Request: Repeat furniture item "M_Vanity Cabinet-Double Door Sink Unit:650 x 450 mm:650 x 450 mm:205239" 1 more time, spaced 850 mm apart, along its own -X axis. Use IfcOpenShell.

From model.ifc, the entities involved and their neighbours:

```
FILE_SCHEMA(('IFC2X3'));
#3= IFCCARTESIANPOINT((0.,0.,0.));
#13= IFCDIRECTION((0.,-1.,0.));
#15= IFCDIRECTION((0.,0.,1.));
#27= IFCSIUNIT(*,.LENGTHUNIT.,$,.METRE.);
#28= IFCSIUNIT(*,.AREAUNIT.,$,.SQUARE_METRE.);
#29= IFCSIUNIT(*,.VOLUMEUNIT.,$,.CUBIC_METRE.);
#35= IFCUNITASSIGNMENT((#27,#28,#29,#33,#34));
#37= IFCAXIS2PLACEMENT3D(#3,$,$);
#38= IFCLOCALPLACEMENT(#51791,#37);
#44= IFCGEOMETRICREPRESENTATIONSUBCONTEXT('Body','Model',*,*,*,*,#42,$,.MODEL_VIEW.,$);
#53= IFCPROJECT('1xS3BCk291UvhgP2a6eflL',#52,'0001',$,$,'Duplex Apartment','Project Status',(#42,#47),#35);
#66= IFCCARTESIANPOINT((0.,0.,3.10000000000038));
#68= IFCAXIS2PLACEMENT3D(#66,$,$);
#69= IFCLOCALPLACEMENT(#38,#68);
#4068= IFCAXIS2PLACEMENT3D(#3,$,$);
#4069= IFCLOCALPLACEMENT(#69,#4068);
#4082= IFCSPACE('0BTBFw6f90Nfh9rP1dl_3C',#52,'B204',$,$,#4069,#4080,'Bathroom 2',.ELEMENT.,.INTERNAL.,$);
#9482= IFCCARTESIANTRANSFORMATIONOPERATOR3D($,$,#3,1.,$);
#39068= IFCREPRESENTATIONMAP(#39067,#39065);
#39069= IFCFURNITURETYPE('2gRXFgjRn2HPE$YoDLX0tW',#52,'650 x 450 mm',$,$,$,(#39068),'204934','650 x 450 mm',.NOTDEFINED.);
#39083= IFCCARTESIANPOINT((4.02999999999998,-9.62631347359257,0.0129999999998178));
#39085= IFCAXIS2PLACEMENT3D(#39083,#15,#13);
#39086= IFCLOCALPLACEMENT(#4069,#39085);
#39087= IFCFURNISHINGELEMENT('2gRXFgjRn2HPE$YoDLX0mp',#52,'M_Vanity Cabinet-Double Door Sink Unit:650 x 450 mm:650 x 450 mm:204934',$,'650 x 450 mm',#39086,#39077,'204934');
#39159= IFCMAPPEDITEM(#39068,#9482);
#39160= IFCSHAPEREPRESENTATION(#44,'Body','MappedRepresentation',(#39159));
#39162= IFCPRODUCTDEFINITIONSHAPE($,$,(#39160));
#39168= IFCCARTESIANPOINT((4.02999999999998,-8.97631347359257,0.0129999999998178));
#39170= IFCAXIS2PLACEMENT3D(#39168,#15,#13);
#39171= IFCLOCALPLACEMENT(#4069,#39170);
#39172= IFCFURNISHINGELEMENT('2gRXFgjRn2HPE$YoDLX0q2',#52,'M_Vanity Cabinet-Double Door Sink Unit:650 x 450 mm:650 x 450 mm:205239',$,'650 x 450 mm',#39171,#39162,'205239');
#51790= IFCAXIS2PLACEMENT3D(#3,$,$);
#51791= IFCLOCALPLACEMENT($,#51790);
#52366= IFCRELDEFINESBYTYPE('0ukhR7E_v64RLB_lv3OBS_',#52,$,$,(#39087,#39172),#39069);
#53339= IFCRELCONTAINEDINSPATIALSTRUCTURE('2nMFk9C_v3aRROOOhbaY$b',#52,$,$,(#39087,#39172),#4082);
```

```python
import ifcopenshell
import ifcopenshell.api.geometry
import ifcopenshell.api.root
import ifcopenshell.util.element
import ifcopenshell.util.placement
import ifcopenshell.util.unit

model = ifcopenshell.open("model.ifc")
unit_scale = ifcopenshell.util.unit.calculate_unit_scale(model)


def reuse_history(source, copy):
    """copy_class also copies each property set's owner history, people and application; keep the originals."""
    for rel in copy.IsDefinedBy:
        if rel.is_a("IfcRelDefinesByProperties") and (history := rel.RelatingPropertyDefinition.OwnerHistory):
            rel.RelatingPropertyDefinition.OwnerHistory = source.OwnerHistory
            ifcopenshell.util.element.remove_deep2(model, history)


source = model.by_guid("2gRXFgjRn2HPE$YoDLX0q2")
base = ifcopenshell.util.placement.get_local_placement(source.ObjectPlacement)
step = -base[:3, 0] * 0.85 / unit_scale

for i in range(1, 2):
    copy = ifcopenshell.api.root.copy_class(model, product=source)
    copy.Representation = ifcopenshell.util.element.copy_deep(
        model, source.Representation, exclude=["IfcGeometricRepresentationContext", "IfcRepresentationMap"]
    )
    copy.Name = "M_Vanity Cabinet-Double Door Sink Unit:650 x 450 mm:650 x 450 mm"
    copy.Tag = None
    reuse_history(source, copy)
    matrix = base.copy()
    matrix[:3, 3] += i * step
    print("added at", matrix[:3, 3].round(3) + 0.0)
    ifcopenshell.api.geometry.edit_object_placement(model, product=copy, matrix=matrix, is_si=False)

model.write("model_edited.ifc")
```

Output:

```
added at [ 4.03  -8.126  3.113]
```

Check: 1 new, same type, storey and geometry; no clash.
